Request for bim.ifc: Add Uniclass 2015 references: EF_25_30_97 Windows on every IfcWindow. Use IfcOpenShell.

First a look at what the model holds.

```python
import ifcopenshell

model = ifcopenshell.open("bim.ifc")
print(model.schema)
print("classifications:", [c.Name for c in model.by_type("IfcClassification")])
for ifc_class in ("IfcDoor", "IfcRoof", "IfcStair", "IfcWall", "IfcWindow"):
    print(ifc_class, len(model.by_type(ifc_class)))
```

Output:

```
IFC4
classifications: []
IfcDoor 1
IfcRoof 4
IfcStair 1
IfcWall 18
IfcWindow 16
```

```python
import ifcopenshell
import ifcopenshell.api.classification

model = ifcopenshell.open("bim.ifc")

system = ifcopenshell.api.classification.add_classification(model, classification="Uniclass 2015")

codes = {
    "IfcWindow": ("EF_25_30_97", "Windows"),
}
for ifc_class, (code, name) in codes.items():
    products = model.by_type(ifc_class)
    ifcopenshell.api.classification.add_reference(
        model, products=products, classification=system, identification=code, name=name
    )
    print(code, len(products))

model.write("bim-out.ifc")
```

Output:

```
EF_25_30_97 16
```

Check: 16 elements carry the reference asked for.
